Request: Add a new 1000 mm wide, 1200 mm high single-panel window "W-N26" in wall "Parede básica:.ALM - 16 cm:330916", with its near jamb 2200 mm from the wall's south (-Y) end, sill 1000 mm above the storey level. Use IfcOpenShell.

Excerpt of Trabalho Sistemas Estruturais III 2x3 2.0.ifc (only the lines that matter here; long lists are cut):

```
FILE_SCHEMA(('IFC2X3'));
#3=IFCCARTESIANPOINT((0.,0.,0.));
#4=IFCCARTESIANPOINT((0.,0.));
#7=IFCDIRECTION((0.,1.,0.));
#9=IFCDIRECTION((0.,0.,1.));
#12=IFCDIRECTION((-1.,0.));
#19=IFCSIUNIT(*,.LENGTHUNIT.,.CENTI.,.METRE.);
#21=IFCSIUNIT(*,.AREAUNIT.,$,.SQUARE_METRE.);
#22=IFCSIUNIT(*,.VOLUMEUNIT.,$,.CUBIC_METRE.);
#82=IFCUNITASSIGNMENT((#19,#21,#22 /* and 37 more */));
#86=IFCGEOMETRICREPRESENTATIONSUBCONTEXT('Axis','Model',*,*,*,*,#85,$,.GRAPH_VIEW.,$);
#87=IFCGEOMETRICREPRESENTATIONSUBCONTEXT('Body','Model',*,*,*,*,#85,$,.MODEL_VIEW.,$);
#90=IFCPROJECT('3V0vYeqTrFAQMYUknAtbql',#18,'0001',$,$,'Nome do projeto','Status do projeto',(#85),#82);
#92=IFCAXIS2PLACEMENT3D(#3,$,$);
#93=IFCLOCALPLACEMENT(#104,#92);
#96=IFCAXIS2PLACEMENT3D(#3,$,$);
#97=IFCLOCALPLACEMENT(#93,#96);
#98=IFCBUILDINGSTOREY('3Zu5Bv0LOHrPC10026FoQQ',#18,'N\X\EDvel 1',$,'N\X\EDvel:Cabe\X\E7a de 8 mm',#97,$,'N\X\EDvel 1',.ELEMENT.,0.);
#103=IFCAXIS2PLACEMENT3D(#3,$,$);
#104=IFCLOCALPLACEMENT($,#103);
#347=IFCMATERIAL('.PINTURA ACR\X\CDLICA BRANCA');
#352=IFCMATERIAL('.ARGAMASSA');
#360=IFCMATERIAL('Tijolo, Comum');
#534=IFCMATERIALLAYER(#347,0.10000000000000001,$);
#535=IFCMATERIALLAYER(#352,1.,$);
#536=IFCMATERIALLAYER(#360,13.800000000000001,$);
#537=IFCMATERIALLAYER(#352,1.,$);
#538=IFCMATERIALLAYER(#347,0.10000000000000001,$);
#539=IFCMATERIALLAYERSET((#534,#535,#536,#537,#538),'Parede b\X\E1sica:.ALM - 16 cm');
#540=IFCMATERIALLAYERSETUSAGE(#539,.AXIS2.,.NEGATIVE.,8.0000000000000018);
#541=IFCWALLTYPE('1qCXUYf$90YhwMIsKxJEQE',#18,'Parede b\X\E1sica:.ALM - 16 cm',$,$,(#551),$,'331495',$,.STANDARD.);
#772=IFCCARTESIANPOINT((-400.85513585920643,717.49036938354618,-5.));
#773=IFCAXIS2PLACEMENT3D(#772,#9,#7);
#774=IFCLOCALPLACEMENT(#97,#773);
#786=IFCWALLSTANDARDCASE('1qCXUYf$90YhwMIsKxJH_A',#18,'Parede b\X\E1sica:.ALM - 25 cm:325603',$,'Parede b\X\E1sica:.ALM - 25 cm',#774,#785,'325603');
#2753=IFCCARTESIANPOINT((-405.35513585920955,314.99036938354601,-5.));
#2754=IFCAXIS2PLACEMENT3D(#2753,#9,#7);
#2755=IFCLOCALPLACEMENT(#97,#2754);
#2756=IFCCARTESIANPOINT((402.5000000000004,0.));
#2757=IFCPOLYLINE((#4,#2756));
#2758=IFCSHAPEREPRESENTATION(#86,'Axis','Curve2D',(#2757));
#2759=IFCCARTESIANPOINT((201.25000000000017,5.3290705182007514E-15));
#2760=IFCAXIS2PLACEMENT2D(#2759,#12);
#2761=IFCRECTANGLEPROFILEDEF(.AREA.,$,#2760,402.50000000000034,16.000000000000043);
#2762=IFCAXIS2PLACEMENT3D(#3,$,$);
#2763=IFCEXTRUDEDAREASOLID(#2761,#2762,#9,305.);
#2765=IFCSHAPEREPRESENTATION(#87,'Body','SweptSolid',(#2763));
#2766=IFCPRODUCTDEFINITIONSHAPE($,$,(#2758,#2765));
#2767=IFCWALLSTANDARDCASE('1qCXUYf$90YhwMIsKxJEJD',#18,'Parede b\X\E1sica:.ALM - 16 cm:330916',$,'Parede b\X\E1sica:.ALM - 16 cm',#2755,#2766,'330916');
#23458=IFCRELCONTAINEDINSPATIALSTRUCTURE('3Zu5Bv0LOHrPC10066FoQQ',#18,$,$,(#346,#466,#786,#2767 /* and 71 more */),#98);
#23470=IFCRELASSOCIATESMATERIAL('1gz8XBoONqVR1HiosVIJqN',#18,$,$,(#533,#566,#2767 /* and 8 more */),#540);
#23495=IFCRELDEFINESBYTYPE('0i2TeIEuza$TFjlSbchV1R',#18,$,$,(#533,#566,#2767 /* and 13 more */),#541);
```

```python
import numpy as np
import ifcopenshell
import ifcopenshell.api.feature
import ifcopenshell.api.geometry
import ifcopenshell.api.root
import ifcopenshell.api.spatial
import ifcopenshell.api.type
import ifcopenshell.geom
import ifcopenshell.util.element
import ifcopenshell.util.placement
import ifcopenshell.util.representation
import ifcopenshell.util.shape
import ifcopenshell.util.unit

model = ifcopenshell.open("Trabalho Sistemas Estruturais III 2x3 2.0.ifc")
unit_scale = ifcopenshell.util.unit.calculate_unit_scale(model)
settings = ifcopenshell.geom.settings()


def volume(element):
    """Net volume in cubic metres, openings subtracted."""
    shape = ifcopenshell.geom.create_shape(settings, element)
    return ifcopenshell.util.shape.get_volume(shape.geometry)


wall = model.by_guid("1qCXUYf$90YhwMIsKxJEJD")
storey = ifcopenshell.util.element.get_container(wall, ifc_class="IfcBuildingStorey")
context = ifcopenshell.util.representation.get_context(model, "Model", "Body", "MODEL_VIEW")
before = volume(wall)

width, height, from_end, sill = 1, 1.2, 2.2, 1  # metres

# The wall runs along its own X axis, and the end named is its -X end.
wall_shape = ifcopenshell.geom.create_shape(settings, wall)
x, y, z = ifcopenshell.util.shape.get_vertices(wall_shape.geometry).T
start = x.min() + from_end
face, thickness = float(y.min()), float(y.max() - y.min())
wall_matrix = ifcopenshell.util.placement.get_local_placement(wall.ObjectPlacement)
level = ifcopenshell.util.placement.get_local_placement(storey.ObjectPlacement)[2, 3]


def in_wall(x, y):
    """Placement at x, y metres in the wall's axes, at sill height."""
    matrix = wall_matrix.copy()
    matrix[:, 3] = wall_matrix @ np.array([x / unit_scale, y / unit_scale, 0.0, 1.0])
    matrix[2, 3] = level + sill / unit_scale
    return matrix


# Opening: a box that overshoots both wall faces by 50 mm.
opening = ifcopenshell.api.root.create_entity(model, ifc_class="IfcOpeningElement")
box = ifcopenshell.api.geometry.add_wall_representation(
    model, context=context, length=width, height=height, thickness=thickness + 0.1
)
ifcopenshell.api.geometry.assign_representation(model, product=opening, representation=box)
ifcopenshell.api.geometry.edit_object_placement(model, product=opening, matrix=in_wall(start, face - 0.05), is_si=False)
ifcopenshell.api.feature.add_feature(model, feature=opening, element=wall)

window = ifcopenshell.api.root.create_entity(model, ifc_class="IfcWindow", name="W-N26")
window.OverallWidth, window.OverallHeight = width / unit_scale, height / unit_scale
body = ifcopenshell.api.geometry.add_window_representation(
    model,
    context=context,
    overall_width=window.OverallWidth,
    overall_height=window.OverallHeight,
    partition_type="SINGLE_PANEL",
)
ifcopenshell.api.geometry.assign_representation(model, product=window, representation=body)
ifcopenshell.api.spatial.assign_container(model, products=[window], relating_structure=storey)
fills = ifcopenshell.api.feature.add_filling(model, opening=opening, element=window)
fills.OwnerHistory = window.OwnerHistory  # required in IFC2X3

# IFC2X3 keeps the operation on the window style.
style = ifcopenshell.api.root.create_entity(model, ifc_class="IfcWindowStyle", name="W-N26")
style.OperationType, style.ConstructionType = "SINGLE_PANEL", "NOTDEFINED"
style.ParameterTakesPrecedence = style.Sizeable = False
ifcopenshell.api.type.assign_type(model, related_objects=[window], relating_type=style)

# Centre the window in the wall's thickness.
ifcopenshell.api.geometry.edit_object_placement(model, product=window, matrix=in_wall(start, face), is_si=False)
window_shape = ifcopenshell.geom.create_shape(settings, window)
depth = ifcopenshell.util.shape.get_vertices(window_shape.geometry)[:, 1]
offset = face + thickness / 2 - (depth.min() + depth.max()) / 2
ifcopenshell.api.geometry.edit_object_placement(model, product=window, matrix=in_wall(start, offset), is_si=False)

after = volume(wall)

print(f"wall volume {before:.3f} -> {after:.3f} m3")

model.write("Trabalho Sistemas Estruturais III 2x3 2.0_updated.ifc")
```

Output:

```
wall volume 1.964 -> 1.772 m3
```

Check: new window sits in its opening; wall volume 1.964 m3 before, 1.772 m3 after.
